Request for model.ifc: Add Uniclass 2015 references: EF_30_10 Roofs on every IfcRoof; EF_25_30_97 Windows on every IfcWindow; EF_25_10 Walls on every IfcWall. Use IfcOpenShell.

First a look at what the model holds.

```python
import ifcopenshell

model = ifcopenshell.open("model.ifc")
print(model.schema)
print("classifications:", [c.Name for c in model.by_type("IfcClassification")])
for ifc_class in ("IfcDoor", "IfcRoof", "IfcStair", "IfcWall", "IfcWindow"):
    print(ifc_class, len(model.by_type(ifc_class)))
```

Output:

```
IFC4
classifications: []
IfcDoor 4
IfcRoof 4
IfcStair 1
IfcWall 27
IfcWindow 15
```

```python
import ifcopenshell
import ifcopenshell.api.classification

model = ifcopenshell.open("model.ifc")

system = ifcopenshell.api.classification.add_classification(model, classification="Uniclass 2015")

codes = {
    "IfcRoof": ("EF_30_10", "Roofs"),
    "IfcWindow": ("EF_25_30_97", "Windows"),
    "IfcWall": ("EF_25_10", "Walls"),
}
for ifc_class, (code, name) in codes.items():
    products = model.by_type(ifc_class)
    ifcopenshell.api.classification.add_reference(
        model, products=products, classification=system, identification=code, name=name
    )
    print(code, len(products))

model.write("model_v2.ifc")
```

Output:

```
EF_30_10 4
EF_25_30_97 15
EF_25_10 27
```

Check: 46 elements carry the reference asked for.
